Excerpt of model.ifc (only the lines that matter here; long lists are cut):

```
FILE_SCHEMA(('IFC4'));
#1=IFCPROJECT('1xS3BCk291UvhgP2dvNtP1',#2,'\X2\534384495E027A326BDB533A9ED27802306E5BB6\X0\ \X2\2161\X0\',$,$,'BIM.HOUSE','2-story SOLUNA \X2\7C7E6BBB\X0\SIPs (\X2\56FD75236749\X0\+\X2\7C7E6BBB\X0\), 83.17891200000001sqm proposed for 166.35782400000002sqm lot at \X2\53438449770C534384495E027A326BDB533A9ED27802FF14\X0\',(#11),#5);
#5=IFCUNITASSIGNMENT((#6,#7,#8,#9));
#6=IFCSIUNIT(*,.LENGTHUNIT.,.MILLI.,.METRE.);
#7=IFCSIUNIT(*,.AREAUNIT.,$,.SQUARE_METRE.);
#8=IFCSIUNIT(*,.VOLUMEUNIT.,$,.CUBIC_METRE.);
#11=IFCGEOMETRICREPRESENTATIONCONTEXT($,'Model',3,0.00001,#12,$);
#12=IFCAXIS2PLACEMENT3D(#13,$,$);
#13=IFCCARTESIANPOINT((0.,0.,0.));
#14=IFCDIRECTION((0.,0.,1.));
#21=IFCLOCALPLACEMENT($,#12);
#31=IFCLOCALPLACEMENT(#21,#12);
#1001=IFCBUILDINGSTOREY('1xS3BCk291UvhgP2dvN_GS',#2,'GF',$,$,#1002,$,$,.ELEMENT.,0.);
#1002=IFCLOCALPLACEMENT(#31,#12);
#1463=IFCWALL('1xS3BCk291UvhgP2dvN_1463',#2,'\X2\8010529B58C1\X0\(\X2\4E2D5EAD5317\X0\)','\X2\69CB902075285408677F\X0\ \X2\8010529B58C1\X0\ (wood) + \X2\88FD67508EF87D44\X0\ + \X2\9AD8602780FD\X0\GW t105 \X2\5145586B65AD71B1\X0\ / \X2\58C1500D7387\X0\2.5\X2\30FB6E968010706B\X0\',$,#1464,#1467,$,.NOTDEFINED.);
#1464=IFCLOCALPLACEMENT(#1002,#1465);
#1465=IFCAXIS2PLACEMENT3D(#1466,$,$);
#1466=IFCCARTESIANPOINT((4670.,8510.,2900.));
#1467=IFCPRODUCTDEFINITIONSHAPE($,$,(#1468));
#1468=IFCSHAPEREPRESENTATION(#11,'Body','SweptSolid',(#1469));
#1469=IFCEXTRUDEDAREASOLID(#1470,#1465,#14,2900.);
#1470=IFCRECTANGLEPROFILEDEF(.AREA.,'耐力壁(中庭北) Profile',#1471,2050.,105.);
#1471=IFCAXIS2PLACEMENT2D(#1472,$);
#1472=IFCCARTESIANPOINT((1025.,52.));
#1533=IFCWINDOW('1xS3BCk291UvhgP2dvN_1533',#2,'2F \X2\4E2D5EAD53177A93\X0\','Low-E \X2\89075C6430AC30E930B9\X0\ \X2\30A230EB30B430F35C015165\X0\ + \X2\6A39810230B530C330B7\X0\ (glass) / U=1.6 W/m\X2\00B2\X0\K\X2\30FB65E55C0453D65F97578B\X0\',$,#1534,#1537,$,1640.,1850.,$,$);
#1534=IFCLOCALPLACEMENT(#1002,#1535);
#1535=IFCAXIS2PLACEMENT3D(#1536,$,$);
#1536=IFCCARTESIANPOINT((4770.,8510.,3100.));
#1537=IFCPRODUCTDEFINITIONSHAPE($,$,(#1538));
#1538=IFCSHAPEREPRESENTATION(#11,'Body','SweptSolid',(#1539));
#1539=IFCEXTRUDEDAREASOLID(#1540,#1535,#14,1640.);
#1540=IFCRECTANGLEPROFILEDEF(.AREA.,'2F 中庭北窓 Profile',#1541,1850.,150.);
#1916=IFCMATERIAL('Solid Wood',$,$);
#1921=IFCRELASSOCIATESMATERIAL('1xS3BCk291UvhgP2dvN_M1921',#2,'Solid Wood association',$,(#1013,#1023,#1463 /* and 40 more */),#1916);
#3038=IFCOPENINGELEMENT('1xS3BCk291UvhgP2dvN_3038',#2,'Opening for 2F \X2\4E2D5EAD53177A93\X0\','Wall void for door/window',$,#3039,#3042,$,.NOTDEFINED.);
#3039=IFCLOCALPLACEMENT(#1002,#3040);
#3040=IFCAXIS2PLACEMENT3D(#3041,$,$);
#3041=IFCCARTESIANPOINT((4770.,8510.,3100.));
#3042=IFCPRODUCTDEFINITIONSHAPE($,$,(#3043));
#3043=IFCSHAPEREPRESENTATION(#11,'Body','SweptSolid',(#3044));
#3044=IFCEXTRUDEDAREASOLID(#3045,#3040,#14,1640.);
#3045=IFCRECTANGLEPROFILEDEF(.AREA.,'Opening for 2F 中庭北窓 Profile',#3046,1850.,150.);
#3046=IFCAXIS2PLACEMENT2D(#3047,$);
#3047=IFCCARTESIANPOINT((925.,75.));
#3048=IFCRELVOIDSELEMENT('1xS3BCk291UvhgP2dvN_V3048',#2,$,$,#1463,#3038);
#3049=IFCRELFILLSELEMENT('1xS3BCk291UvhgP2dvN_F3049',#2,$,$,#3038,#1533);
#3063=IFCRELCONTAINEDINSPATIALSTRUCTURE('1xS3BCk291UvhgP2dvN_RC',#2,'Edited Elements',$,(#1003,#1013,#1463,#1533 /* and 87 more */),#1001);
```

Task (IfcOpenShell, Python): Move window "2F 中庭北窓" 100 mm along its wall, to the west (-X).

```python
import ifcopenshell
import ifcopenshell.api.geometry
import ifcopenshell.util.placement
import ifcopenshell.util.unit

model = ifcopenshell.open("model.ifc")
unit_scale = ifcopenshell.util.unit.calculate_unit_scale(model)

window = model.by_guid("1xS3BCk291UvhgP2dvN_1533")
opening = window.FillsVoids[0].RelatingOpeningElement
wall = opening.VoidsElements[0].RelatingBuildingElement

wall_matrix = ifcopenshell.util.placement.get_local_placement(wall.ObjectPlacement)
shift = wall_matrix[:3, 0] * -0.1 / unit_scale
before = ifcopenshell.util.placement.get_local_placement(window.ObjectPlacement)[:3, 3].copy()

# The window is not placed relative to its opening, so move both.
for product in (opening, window):
    matrix = ifcopenshell.util.placement.get_local_placement(product.ObjectPlacement)
    matrix[:3, 3] += shift
    ifcopenshell.api.geometry.edit_object_placement(model, product=product, matrix=matrix, is_si=False)

after = ifcopenshell.util.placement.get_local_placement(window.ObjectPlacement)[:3, 3]
print("window moved by", (after - before).round(3) + 0.0)

model.write("model_updated.ifc")
```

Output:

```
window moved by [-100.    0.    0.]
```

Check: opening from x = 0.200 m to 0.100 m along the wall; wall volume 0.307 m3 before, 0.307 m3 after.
